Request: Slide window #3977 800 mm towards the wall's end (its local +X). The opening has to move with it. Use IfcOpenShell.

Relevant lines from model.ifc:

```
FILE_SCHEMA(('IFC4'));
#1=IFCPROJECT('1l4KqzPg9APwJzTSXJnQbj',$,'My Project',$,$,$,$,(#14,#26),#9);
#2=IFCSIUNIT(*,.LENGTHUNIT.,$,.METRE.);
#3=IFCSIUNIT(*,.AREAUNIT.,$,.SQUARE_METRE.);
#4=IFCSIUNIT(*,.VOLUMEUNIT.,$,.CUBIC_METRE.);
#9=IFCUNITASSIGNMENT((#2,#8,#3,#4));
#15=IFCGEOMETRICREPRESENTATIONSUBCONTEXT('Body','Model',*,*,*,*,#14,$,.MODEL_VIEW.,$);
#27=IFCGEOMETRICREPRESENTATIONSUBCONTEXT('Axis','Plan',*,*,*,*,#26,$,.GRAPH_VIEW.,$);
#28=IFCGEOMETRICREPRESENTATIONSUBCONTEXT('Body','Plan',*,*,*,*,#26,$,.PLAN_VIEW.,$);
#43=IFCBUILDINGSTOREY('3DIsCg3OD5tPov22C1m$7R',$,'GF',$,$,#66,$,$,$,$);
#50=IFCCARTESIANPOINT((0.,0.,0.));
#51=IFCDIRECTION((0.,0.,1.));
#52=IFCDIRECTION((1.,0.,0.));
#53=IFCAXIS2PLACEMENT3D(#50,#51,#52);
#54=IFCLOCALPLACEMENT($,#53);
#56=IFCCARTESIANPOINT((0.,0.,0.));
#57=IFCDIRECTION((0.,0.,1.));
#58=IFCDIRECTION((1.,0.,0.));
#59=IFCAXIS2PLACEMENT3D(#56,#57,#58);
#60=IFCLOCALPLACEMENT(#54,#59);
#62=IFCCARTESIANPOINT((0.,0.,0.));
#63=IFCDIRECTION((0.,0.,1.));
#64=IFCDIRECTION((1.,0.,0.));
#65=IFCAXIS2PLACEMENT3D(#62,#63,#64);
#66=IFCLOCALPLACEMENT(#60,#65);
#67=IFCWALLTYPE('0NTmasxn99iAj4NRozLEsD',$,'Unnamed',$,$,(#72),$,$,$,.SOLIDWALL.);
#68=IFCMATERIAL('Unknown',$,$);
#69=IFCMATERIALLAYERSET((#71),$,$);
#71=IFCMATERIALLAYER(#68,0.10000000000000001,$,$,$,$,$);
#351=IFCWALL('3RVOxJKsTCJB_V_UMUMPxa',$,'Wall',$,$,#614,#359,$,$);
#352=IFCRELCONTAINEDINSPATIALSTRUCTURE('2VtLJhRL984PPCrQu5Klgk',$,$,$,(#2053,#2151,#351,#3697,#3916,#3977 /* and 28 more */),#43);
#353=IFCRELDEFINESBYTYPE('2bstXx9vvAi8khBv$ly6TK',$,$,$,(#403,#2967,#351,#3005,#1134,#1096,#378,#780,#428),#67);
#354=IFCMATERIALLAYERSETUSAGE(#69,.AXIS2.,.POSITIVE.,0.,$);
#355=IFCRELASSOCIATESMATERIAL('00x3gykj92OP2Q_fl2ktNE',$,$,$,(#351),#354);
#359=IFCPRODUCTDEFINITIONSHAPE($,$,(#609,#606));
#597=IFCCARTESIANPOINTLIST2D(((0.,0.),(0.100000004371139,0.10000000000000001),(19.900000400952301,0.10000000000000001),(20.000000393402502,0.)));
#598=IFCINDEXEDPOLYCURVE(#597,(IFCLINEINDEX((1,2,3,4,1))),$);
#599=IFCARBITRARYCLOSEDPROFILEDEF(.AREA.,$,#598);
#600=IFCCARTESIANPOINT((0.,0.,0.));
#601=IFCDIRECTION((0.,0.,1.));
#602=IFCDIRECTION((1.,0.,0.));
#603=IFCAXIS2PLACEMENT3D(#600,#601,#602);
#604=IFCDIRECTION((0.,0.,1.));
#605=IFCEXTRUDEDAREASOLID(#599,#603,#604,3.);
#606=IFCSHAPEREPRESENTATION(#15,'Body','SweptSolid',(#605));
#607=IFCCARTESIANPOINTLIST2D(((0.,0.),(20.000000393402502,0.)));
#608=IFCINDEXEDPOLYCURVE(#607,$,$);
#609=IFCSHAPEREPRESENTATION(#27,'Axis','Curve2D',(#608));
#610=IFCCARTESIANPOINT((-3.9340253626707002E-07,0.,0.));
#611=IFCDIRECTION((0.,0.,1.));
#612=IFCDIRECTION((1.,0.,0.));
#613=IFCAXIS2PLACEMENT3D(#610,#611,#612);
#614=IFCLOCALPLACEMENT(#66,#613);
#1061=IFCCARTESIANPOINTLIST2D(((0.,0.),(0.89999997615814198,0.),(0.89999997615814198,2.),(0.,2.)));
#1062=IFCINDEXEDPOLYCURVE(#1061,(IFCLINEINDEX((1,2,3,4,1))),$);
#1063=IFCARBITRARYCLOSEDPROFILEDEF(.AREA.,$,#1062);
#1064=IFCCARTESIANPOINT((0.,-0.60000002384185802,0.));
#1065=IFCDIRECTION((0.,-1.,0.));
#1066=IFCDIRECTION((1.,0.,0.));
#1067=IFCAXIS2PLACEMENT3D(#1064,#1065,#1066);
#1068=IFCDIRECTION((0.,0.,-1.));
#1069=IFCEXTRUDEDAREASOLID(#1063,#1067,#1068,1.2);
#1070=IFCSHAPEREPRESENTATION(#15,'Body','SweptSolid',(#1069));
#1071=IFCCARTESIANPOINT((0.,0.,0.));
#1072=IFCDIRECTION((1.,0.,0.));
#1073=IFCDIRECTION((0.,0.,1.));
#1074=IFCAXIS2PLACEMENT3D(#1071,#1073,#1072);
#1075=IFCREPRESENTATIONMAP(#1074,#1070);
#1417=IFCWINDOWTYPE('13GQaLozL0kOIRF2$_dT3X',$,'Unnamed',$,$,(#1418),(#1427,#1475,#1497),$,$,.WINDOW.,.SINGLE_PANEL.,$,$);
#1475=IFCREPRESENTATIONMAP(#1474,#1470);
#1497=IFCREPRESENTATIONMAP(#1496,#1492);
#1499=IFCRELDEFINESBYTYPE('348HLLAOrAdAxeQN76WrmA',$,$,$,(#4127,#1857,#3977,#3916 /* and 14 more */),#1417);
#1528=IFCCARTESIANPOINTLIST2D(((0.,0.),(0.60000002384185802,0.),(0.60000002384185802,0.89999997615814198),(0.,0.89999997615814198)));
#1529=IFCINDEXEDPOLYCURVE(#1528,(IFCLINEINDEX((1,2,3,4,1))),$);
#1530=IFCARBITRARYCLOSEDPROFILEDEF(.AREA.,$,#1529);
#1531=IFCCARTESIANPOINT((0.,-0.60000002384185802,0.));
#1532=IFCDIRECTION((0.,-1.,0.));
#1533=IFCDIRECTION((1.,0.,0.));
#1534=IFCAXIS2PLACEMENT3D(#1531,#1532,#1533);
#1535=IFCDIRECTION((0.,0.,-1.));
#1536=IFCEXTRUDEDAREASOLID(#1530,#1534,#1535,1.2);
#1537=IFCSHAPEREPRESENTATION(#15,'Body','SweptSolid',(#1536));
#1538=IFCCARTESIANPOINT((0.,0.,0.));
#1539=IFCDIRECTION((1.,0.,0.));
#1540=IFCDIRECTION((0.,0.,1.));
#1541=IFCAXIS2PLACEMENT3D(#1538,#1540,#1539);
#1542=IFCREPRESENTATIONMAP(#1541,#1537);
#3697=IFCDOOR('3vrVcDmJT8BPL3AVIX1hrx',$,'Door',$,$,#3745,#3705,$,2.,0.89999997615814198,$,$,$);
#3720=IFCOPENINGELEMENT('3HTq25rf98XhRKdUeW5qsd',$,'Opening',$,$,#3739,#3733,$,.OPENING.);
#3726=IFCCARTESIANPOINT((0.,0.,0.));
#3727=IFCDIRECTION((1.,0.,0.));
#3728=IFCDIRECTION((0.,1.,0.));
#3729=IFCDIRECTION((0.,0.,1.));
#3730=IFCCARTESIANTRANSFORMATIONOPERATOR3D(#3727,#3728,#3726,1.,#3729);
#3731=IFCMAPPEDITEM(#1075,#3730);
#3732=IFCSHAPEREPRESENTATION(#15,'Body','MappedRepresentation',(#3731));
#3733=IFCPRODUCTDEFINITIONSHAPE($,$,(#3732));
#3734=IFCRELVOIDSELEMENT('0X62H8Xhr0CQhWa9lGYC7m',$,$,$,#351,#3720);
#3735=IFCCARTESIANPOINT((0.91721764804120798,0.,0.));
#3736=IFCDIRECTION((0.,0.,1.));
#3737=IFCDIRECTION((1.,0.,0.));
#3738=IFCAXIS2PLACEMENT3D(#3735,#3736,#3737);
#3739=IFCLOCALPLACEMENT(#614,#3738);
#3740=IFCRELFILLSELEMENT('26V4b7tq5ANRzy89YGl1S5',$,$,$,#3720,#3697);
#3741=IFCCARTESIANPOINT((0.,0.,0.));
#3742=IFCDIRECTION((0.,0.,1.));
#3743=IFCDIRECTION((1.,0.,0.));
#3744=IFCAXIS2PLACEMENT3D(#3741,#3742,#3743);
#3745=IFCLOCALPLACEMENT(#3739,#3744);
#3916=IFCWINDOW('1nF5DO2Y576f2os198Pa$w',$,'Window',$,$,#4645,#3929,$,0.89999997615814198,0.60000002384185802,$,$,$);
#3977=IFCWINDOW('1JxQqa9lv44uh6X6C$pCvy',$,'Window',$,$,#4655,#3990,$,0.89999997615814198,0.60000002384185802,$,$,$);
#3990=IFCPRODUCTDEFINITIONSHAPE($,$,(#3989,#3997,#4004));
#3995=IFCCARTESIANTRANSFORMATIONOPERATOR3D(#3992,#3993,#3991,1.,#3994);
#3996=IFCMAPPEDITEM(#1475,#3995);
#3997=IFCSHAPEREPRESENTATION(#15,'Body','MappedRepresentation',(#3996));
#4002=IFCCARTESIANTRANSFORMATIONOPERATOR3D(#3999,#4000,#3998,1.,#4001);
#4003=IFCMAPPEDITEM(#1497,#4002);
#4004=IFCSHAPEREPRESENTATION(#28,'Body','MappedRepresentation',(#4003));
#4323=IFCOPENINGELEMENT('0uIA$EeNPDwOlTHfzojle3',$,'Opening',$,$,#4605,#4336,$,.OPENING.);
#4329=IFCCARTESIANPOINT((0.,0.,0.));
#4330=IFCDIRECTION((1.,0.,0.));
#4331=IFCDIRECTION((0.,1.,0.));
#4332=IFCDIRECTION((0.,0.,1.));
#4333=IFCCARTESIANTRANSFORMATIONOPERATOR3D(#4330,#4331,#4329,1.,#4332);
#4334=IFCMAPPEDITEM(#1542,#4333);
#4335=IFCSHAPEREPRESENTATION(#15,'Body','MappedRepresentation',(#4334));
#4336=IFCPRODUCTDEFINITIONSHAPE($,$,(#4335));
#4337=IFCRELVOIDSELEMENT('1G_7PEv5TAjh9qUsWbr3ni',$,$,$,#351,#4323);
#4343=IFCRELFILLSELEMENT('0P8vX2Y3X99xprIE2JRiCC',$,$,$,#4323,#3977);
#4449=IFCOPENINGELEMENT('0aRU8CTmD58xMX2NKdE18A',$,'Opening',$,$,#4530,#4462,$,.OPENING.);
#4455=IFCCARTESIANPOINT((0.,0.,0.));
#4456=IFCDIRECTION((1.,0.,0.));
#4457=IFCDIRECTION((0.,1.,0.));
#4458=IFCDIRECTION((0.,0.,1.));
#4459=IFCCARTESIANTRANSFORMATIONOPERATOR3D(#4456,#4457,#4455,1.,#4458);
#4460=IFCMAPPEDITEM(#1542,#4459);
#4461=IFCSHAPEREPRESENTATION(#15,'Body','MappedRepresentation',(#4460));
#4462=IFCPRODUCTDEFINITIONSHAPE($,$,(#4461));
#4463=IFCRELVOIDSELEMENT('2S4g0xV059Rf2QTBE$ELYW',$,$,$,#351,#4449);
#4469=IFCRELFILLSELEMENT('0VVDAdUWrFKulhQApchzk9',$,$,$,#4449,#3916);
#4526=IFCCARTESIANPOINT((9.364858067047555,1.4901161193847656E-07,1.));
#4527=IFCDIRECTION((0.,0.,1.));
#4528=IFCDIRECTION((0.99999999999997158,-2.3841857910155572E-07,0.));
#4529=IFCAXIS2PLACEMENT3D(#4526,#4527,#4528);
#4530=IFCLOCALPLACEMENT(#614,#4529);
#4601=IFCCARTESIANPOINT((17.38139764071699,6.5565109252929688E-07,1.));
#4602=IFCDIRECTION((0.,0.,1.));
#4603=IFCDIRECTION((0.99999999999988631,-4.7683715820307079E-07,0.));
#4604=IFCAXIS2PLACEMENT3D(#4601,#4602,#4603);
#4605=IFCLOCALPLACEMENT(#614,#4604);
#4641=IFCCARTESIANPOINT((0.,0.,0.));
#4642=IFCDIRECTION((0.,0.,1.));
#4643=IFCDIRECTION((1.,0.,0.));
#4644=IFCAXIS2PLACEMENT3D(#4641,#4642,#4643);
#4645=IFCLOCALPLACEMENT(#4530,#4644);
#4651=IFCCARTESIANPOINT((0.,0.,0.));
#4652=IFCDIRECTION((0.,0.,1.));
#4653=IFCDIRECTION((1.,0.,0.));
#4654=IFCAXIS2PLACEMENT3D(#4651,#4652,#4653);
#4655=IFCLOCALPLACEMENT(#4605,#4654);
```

```python
import ifcopenshell
import ifcopenshell.api.geometry
import ifcopenshell.util.placement
import ifcopenshell.util.unit

model = ifcopenshell.open("model.ifc")
unit_scale = ifcopenshell.util.unit.calculate_unit_scale(model)

window = model.by_id(3977)
opening = window.FillsVoids[0].RelatingOpeningElement
wall = opening.VoidsElements[0].RelatingBuildingElement

wall_matrix = ifcopenshell.util.placement.get_local_placement(wall.ObjectPlacement)
shift = wall_matrix[:3, 0] * 0.8 / unit_scale
before = ifcopenshell.util.placement.get_local_placement(window.ObjectPlacement)[:3, 3].copy()

# The window is placed relative to its opening, so it follows when the opening moves.
matrix = ifcopenshell.util.placement.get_local_placement(opening.ObjectPlacement)
matrix[:3, 3] += shift
ifcopenshell.api.geometry.edit_object_placement(
    model, product=opening, matrix=matrix, is_si=False, should_transform_children=True
)

after = ifcopenshell.util.placement.get_local_placement(window.ObjectPlacement)[:3, 3]
print("window moved by", (after - before).round(3) + 0.0)

model.write("model-out.ifc")
```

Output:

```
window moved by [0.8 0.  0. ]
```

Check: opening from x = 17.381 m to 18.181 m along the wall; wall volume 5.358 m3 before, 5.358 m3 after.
